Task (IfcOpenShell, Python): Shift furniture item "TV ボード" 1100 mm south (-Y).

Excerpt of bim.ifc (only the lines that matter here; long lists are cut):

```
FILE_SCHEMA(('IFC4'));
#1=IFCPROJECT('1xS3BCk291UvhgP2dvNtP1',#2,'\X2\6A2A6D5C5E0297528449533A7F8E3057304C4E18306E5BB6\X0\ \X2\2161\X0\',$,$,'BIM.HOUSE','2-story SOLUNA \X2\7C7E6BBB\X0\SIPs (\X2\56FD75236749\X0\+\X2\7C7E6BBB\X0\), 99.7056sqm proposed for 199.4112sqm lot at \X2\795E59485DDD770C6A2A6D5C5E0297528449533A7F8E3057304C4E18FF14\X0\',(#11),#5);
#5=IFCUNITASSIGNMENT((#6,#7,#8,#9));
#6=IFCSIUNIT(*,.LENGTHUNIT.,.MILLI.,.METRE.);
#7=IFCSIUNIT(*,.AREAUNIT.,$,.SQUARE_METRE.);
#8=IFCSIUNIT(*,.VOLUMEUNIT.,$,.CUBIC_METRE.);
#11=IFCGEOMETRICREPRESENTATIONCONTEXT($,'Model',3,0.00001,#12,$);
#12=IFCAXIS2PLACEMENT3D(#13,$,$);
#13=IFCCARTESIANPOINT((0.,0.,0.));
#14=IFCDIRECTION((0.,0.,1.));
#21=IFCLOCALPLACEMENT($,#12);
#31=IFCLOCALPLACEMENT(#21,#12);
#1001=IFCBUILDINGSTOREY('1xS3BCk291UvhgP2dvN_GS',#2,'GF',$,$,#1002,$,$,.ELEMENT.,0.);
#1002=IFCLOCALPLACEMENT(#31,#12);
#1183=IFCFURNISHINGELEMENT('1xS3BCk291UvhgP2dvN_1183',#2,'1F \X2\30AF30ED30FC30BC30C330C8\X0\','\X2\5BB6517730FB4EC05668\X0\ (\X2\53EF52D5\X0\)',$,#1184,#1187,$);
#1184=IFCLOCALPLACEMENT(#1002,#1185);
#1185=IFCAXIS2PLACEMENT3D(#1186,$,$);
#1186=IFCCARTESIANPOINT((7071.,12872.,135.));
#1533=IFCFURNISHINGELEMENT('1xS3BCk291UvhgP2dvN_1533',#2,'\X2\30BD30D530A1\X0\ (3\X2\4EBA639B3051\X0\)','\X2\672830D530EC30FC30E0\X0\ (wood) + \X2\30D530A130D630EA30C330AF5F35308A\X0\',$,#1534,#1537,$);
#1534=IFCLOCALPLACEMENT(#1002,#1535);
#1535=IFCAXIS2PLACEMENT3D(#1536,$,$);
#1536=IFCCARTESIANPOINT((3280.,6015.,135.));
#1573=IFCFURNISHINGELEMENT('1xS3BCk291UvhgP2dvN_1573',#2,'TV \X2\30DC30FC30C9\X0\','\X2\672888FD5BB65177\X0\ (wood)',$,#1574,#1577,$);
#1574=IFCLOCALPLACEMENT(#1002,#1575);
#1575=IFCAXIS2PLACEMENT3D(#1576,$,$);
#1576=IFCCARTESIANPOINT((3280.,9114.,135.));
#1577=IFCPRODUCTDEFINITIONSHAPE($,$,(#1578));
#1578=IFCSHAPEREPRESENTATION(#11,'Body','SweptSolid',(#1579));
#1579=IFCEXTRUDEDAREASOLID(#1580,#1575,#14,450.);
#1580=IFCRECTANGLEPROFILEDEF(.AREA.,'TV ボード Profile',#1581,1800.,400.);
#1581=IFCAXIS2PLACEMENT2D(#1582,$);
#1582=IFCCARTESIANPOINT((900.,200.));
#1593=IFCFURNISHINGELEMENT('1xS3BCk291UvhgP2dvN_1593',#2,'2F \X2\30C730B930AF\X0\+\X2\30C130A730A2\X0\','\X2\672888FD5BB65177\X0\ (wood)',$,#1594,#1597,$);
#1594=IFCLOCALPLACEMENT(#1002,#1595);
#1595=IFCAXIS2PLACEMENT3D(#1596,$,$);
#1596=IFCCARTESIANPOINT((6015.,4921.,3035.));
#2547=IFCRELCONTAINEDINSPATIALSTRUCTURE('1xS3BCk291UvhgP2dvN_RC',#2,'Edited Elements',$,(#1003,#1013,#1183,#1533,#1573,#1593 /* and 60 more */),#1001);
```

```python
import ifcopenshell
import ifcopenshell.api.geometry
import ifcopenshell.util.placement
import ifcopenshell.util.unit

model = ifcopenshell.open("bim.ifc")
unit_scale = ifcopenshell.util.unit.calculate_unit_scale(model)

item = model.by_id(1573)
matrix = ifcopenshell.util.placement.get_local_placement(item.ObjectPlacement)
matrix[1, 3] -= 1.1 / unit_scale
ifcopenshell.api.geometry.edit_object_placement(model, product=item, matrix=matrix, is_si=False)

print(ifcopenshell.util.placement.get_local_placement(item.ObjectPlacement).round(3) + 0.0)

model.write("bim_updated.ifc")
```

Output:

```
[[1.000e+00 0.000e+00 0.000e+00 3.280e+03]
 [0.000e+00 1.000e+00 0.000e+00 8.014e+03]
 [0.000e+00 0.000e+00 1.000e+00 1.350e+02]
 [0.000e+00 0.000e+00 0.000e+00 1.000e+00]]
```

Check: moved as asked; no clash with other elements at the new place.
